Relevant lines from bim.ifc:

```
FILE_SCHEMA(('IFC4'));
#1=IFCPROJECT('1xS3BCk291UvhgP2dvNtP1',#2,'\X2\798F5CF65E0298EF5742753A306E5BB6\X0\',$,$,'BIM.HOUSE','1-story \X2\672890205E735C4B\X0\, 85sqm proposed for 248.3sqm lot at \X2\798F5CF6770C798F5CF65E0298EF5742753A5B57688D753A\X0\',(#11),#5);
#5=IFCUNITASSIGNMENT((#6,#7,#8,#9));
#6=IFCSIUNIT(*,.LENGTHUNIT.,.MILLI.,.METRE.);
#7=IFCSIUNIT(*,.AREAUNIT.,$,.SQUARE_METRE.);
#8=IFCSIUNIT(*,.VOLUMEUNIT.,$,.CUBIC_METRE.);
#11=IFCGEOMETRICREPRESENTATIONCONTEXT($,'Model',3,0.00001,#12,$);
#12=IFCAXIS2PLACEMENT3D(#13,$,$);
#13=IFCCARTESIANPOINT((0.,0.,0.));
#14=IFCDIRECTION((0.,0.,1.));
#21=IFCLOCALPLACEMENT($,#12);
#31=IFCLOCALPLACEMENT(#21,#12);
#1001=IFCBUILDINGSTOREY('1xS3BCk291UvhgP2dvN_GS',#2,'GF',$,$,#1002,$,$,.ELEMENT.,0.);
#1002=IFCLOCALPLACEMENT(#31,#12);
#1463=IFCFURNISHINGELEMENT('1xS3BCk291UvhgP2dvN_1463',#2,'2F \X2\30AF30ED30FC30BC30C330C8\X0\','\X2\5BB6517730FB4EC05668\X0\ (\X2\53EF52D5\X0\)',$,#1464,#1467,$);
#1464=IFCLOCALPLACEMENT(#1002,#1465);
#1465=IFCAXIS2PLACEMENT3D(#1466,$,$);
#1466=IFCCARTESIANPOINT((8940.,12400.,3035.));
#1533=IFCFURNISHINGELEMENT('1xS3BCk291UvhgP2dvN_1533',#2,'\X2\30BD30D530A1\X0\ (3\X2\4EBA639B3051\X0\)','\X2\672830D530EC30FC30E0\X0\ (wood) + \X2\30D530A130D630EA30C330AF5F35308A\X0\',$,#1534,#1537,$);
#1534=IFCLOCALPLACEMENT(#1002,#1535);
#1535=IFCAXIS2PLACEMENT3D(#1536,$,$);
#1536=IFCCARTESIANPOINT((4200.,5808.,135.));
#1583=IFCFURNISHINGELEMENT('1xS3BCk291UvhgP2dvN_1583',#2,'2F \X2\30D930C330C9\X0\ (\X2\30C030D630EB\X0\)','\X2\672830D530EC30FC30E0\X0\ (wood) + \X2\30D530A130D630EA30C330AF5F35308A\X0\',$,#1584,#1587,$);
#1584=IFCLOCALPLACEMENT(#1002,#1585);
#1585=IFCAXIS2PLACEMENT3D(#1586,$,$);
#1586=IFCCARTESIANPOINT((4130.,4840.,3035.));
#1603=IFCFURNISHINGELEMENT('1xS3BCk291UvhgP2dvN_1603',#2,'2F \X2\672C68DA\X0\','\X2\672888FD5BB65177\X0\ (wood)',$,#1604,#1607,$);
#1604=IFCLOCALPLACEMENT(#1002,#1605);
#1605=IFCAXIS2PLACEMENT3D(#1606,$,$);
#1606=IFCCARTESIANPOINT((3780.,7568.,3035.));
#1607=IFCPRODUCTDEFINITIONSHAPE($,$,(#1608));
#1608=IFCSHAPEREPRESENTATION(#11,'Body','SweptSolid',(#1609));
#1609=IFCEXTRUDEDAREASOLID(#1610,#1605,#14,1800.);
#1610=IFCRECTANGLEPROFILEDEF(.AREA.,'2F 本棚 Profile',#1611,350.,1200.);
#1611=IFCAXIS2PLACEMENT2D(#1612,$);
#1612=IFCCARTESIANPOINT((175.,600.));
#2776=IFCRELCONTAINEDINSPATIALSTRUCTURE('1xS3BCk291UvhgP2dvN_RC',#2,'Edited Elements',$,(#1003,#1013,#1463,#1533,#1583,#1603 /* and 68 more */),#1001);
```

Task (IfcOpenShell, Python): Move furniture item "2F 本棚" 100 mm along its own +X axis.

```python
import ifcopenshell
import ifcopenshell.api.geometry
import ifcopenshell.util.placement
import ifcopenshell.util.unit

model = ifcopenshell.open("bim.ifc")
unit_scale = ifcopenshell.util.unit.calculate_unit_scale(model)

item = model.by_id(1603)
matrix = ifcopenshell.util.placement.get_local_placement(item.ObjectPlacement)
matrix[:3, 3] += matrix[:3, 0] * 0.1 / unit_scale
ifcopenshell.api.geometry.edit_object_placement(model, product=item, matrix=matrix, is_si=False)

print(ifcopenshell.util.placement.get_local_placement(item.ObjectPlacement).round(3) + 0.0)

model.write("bim_updated.ifc")
```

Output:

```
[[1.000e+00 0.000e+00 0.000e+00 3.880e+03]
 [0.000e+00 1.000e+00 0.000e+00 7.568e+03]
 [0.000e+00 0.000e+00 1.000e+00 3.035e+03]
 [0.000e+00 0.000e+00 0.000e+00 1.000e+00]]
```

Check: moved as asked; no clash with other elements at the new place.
